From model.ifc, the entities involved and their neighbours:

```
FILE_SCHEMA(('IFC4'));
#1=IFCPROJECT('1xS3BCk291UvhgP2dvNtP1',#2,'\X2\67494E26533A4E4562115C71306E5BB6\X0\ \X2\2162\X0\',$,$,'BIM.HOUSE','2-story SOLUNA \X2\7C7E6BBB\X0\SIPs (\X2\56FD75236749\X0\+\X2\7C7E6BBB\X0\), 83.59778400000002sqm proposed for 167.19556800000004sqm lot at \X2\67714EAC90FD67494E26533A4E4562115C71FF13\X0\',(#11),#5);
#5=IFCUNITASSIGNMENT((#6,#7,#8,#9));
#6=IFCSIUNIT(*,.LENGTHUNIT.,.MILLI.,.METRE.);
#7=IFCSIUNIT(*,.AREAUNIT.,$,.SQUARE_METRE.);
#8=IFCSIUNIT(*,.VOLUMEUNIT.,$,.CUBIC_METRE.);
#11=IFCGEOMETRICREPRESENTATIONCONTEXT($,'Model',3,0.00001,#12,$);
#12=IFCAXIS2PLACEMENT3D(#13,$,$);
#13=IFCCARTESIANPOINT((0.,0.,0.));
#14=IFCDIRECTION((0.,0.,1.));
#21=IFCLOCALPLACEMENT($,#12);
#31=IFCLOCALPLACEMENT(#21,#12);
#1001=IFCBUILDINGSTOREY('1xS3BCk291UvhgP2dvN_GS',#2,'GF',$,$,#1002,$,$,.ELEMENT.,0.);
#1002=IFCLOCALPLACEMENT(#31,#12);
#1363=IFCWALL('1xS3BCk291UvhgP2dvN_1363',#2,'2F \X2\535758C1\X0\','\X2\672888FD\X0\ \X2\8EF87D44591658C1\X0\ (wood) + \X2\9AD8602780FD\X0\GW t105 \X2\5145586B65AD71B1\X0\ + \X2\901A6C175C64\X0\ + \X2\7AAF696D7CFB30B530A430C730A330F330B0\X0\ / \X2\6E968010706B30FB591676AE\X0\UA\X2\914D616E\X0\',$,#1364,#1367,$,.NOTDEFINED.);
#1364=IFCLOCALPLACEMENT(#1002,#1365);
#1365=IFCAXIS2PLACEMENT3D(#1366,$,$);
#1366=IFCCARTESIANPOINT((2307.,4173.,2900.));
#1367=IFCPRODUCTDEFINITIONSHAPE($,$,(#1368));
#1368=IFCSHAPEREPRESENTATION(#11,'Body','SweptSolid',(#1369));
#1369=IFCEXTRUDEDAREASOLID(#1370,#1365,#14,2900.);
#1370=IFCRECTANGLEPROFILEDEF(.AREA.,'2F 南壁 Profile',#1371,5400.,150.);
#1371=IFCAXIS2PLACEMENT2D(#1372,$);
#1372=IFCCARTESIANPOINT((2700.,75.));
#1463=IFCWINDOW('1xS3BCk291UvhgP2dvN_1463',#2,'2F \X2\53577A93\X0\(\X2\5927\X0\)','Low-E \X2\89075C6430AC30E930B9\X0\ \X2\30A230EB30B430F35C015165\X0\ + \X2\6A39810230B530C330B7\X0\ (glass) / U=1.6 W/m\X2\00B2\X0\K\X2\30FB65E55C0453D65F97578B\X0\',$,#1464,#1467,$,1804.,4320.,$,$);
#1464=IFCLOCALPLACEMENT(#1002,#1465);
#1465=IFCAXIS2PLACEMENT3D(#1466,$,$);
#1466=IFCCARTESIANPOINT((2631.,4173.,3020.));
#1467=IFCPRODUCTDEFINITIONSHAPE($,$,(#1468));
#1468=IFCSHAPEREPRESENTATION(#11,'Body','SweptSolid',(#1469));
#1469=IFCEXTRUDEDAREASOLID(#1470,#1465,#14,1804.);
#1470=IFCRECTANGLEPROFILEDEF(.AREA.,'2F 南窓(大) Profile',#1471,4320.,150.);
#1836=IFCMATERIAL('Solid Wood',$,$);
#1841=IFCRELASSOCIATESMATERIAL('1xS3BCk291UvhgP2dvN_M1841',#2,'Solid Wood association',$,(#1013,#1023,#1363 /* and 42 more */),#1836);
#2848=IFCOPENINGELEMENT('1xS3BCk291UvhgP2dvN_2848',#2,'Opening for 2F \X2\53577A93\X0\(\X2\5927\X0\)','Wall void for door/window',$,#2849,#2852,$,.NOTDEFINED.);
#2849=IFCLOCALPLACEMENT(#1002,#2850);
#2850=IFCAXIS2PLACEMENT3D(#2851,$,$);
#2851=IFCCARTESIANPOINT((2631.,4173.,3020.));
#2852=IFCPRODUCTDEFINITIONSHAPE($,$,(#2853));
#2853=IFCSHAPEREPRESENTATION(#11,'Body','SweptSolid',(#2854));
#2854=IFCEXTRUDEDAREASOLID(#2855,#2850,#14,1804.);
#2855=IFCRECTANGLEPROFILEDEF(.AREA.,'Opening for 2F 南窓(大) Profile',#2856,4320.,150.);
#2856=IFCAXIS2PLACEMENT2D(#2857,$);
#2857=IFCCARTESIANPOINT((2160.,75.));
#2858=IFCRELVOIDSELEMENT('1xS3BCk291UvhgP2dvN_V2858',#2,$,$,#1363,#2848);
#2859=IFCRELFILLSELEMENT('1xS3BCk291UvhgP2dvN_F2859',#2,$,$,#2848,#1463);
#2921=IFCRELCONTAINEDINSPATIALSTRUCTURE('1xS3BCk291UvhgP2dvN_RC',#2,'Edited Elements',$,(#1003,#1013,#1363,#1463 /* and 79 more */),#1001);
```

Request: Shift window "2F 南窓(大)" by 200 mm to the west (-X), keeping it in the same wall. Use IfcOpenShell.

```python
import ifcopenshell
import ifcopenshell.api.geometry
import ifcopenshell.util.placement

model = ifcopenshell.open("model.ifc")

window = model.by_id(1463)
opening = window.FillsVoids[0].RelatingOpeningElement
wall = opening.VoidsElements[0].RelatingBuildingElement

wall_matrix = ifcopenshell.util.placement.get_local_placement(wall.ObjectPlacement)
shift = wall_matrix[:3, 0] * -200.0
before = ifcopenshell.util.placement.get_local_placement(window.ObjectPlacement)[:3, 3].copy()

# The window is not placed relative to its opening, so move both.
for product in (opening, window):
    matrix = ifcopenshell.util.placement.get_local_placement(product.ObjectPlacement)
    matrix[:3, 3] += shift
    ifcopenshell.api.geometry.edit_object_placement(model, product=product, matrix=matrix, is_si=False)

after = ifcopenshell.util.placement.get_local_placement(window.ObjectPlacement)[:3, 3]
print("window moved by", (after - before).round(3) + 0.0)

model.write("model-out.ifc")
```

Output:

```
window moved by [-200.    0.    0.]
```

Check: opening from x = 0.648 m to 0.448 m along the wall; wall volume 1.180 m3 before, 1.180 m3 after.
